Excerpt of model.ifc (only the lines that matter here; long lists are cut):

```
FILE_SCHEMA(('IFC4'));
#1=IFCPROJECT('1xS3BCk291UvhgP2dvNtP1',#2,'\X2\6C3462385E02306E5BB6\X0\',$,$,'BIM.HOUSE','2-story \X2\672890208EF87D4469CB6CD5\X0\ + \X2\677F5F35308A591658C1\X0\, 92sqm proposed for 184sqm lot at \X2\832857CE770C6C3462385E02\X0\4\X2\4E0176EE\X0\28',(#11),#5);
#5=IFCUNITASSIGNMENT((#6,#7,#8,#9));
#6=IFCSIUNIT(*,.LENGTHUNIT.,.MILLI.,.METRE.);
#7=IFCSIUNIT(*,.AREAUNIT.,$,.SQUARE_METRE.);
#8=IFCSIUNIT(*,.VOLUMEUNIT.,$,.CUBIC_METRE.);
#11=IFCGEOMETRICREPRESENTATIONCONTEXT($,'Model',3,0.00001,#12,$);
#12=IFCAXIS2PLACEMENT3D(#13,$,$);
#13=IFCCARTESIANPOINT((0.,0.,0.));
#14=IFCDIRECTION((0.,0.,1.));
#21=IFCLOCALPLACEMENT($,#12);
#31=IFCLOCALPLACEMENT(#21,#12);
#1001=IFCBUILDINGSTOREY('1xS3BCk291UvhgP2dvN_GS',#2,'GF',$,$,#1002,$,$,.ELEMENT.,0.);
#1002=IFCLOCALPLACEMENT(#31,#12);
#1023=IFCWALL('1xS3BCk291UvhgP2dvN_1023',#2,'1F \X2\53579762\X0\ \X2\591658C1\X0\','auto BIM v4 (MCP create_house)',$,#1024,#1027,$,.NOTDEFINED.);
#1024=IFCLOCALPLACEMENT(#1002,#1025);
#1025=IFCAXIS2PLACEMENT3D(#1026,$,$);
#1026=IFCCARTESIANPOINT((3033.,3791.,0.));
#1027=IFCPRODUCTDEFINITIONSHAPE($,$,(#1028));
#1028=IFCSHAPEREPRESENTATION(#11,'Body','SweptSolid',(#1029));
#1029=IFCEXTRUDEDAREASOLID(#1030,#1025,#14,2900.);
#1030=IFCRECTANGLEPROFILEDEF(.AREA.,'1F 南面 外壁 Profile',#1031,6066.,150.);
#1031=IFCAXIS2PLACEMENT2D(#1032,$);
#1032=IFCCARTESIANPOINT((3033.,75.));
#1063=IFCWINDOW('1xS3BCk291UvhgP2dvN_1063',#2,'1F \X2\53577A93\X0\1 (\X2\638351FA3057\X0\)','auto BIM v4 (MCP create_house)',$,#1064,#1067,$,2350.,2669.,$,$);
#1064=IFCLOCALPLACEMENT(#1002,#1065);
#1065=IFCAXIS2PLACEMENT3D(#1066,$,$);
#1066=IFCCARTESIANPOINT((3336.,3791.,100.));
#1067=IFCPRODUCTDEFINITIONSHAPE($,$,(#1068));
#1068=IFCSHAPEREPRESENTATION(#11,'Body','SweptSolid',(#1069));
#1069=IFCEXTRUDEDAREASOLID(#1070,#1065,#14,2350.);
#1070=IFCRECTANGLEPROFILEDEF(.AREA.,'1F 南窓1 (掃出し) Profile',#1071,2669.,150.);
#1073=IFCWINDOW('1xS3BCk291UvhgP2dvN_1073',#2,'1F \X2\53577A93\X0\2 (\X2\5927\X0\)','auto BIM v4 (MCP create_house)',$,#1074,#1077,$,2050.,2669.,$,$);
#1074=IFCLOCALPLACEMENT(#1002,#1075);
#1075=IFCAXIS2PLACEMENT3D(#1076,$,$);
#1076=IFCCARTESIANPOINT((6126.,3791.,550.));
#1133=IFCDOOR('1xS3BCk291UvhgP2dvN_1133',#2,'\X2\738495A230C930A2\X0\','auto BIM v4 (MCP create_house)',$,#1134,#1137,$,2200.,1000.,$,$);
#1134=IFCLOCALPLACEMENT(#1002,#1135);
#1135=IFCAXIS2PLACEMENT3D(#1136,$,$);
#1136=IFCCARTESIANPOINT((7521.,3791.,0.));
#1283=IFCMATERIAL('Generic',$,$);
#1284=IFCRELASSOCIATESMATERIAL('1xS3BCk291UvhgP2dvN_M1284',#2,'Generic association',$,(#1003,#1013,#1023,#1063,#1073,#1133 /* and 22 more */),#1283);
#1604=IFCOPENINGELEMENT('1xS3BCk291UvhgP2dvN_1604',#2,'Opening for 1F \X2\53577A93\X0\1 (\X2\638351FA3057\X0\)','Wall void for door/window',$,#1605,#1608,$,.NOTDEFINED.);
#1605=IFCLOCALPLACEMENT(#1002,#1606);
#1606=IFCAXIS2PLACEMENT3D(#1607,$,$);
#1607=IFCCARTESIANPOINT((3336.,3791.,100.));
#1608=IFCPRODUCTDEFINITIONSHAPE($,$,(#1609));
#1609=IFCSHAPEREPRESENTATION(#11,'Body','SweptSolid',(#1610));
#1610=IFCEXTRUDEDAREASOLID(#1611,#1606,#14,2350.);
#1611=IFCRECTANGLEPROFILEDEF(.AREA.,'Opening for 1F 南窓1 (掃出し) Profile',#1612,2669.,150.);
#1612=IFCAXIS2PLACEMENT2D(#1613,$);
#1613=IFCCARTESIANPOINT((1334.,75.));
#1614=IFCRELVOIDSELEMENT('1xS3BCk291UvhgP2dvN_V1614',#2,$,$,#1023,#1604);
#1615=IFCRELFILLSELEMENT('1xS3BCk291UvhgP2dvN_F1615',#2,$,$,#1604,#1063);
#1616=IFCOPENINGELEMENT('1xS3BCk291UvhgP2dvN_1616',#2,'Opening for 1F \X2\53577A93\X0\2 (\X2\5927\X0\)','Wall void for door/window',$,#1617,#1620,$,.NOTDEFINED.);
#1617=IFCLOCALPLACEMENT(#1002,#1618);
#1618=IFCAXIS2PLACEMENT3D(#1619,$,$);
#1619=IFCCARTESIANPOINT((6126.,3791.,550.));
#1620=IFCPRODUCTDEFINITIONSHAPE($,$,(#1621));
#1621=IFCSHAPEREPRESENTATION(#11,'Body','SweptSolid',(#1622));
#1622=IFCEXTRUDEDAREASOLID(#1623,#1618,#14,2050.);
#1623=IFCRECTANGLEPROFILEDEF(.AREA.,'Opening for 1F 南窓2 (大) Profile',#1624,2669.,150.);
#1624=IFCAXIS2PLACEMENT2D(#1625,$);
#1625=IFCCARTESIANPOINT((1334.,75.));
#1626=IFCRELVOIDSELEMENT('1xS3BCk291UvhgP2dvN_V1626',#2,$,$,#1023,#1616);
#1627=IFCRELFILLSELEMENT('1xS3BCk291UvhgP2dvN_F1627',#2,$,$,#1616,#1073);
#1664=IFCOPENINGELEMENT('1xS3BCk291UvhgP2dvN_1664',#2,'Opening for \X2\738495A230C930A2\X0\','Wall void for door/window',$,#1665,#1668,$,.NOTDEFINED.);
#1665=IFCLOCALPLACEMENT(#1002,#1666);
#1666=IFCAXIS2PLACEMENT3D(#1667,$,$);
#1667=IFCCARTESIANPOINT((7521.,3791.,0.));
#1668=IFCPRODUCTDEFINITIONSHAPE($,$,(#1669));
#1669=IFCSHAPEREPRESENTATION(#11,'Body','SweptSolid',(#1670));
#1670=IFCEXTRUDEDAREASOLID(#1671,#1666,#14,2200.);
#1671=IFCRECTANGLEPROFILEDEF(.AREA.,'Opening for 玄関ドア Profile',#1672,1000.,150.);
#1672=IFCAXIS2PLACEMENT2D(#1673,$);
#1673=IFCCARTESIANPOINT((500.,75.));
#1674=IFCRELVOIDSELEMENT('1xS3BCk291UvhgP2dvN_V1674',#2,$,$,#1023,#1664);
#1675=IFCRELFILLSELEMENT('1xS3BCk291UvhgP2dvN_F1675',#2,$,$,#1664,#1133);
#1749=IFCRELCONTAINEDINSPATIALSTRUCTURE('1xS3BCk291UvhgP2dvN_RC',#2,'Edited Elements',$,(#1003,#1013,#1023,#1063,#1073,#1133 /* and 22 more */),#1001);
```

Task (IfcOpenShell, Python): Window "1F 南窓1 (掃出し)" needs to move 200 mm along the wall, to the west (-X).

```python
import ifcopenshell
import ifcopenshell.api.geometry
import ifcopenshell.util.placement

model = ifcopenshell.open("model.ifc")

window = model.by_guid("1xS3BCk291UvhgP2dvN_1063")
opening = window.FillsVoids[0].RelatingOpeningElement
wall = opening.VoidsElements[0].RelatingBuildingElement

wall_matrix = ifcopenshell.util.placement.get_local_placement(wall.ObjectPlacement)
shift = wall_matrix[:3, 0] * -200.0
before = ifcopenshell.util.placement.get_local_placement(window.ObjectPlacement)[:3, 3].copy()

# The window is not placed relative to its opening, so move both.
for product in (opening, window):
    matrix = ifcopenshell.util.placement.get_local_placement(product.ObjectPlacement)
    matrix[:3, 3] += shift
    ifcopenshell.api.geometry.edit_object_placement(model, product=product, matrix=matrix, is_si=False)

after = ifcopenshell.util.placement.get_local_placement(window.ObjectPlacement)[:3, 3]
print("window moved by", (after - before).round(3) + 0.0)

model.write("model_v2.ifc")
```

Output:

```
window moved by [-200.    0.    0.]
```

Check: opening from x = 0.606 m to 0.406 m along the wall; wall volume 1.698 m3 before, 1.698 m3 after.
